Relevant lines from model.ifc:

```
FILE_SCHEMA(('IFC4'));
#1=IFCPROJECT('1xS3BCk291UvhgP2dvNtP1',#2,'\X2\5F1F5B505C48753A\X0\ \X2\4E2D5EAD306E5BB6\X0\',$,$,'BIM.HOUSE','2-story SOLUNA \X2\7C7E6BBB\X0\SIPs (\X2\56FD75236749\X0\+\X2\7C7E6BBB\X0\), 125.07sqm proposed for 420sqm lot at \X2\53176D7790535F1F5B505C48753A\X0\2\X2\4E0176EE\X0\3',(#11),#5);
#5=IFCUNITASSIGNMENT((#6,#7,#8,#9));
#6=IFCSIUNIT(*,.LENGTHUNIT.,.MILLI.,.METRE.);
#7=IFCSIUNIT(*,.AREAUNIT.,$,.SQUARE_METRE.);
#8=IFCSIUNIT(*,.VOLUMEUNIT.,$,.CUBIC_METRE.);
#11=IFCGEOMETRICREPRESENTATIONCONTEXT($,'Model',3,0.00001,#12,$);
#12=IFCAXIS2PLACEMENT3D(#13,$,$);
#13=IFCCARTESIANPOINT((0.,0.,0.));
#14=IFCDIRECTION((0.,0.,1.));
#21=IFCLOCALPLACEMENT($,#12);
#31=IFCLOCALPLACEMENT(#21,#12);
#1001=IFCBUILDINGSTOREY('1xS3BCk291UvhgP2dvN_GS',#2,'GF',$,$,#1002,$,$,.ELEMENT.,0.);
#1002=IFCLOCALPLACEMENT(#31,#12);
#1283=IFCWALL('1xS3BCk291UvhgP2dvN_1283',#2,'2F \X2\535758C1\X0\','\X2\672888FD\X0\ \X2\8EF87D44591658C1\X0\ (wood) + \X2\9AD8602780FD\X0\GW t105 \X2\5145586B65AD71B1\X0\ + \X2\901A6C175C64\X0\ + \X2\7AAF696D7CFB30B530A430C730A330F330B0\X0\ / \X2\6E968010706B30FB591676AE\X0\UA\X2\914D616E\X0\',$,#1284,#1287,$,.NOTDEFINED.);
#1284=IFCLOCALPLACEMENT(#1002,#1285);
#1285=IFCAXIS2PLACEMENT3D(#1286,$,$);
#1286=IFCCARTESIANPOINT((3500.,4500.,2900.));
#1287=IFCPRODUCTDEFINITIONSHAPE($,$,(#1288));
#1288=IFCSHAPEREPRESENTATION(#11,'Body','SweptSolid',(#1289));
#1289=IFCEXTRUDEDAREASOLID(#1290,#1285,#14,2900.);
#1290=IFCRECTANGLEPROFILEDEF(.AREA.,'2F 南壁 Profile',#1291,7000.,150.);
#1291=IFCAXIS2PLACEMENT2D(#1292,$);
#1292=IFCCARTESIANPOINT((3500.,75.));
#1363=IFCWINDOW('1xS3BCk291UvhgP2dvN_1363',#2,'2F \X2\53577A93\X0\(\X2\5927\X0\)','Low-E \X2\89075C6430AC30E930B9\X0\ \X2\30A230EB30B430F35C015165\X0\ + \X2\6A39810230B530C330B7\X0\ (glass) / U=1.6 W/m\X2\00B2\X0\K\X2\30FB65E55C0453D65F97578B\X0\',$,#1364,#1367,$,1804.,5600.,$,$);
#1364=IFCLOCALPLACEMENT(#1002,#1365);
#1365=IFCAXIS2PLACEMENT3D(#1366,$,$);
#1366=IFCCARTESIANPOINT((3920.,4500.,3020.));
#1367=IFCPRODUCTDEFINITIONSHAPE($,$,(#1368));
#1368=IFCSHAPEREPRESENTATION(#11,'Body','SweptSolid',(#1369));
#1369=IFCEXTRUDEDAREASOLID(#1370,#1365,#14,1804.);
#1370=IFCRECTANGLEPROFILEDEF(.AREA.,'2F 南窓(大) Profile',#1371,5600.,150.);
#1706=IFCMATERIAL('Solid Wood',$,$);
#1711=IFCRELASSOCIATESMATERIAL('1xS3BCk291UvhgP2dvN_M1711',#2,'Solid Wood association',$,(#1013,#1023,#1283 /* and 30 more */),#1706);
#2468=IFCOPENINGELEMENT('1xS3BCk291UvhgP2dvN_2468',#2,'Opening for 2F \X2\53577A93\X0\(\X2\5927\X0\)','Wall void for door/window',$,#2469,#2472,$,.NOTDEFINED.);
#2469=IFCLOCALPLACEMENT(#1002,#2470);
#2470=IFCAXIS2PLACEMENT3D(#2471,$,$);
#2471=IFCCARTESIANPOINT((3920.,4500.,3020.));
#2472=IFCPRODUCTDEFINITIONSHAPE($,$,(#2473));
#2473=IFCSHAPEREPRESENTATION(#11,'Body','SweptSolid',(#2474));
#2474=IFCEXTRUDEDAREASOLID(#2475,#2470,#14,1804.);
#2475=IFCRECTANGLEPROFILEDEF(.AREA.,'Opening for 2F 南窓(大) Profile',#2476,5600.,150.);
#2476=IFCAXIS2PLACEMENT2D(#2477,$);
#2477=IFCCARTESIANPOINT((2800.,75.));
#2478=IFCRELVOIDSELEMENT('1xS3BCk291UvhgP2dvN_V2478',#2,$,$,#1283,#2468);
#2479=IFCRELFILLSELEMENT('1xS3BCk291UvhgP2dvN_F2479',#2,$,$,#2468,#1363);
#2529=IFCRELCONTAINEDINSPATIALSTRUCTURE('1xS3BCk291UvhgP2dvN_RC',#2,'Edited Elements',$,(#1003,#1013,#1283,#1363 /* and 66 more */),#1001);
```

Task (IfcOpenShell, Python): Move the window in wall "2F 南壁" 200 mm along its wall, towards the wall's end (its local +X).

```python
import ifcopenshell
import ifcopenshell.api.geometry
import ifcopenshell.util.placement
import ifcopenshell.util.unit

model = ifcopenshell.open("model.ifc")
unit_scale = ifcopenshell.util.unit.calculate_unit_scale(model)

window = model.by_guid("1xS3BCk291UvhgP2dvN_1363")
opening = window.FillsVoids[0].RelatingOpeningElement
wall = opening.VoidsElements[0].RelatingBuildingElement

wall_matrix = ifcopenshell.util.placement.get_local_placement(wall.ObjectPlacement)
shift = wall_matrix[:3, 0] * 0.2 / unit_scale
before = ifcopenshell.util.placement.get_local_placement(window.ObjectPlacement)[:3, 3].copy()

# The window is not placed relative to its opening, so move both.
for product in (opening, window):
    matrix = ifcopenshell.util.placement.get_local_placement(product.ObjectPlacement)
    matrix[:3, 3] += shift
    ifcopenshell.api.geometry.edit_object_placement(model, product=product, matrix=matrix, is_si=False)

after = ifcopenshell.util.placement.get_local_placement(window.ObjectPlacement)[:3, 3]
print("window moved by", (after - before).round(3) + 0.0)

model.write("model_updated.ifc")
```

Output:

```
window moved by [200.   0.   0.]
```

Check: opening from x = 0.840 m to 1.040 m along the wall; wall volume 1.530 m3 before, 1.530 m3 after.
